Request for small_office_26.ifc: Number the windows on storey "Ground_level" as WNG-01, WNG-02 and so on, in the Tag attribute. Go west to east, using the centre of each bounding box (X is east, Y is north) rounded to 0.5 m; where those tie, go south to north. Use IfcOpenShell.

First a look at what the model holds.

```python
import ifcopenshell
import ifcopenshell.util.element
import ifcopenshell.util.placement

model = ifcopenshell.open("small_office_26.ifc")
print(model.schema)
storey = next(s for s in model.by_type("IfcBuildingStorey") if s.Name == "Ground_level")
windows = [e for e in ifcopenshell.util.element.get_decomposition(storey) if e.is_a("IfcWindow")]
for e in sorted(windows, key=lambda e: e.id()):
    origin = ifcopenshell.util.placement.get_local_placement(e.ObjectPlacement)[:3, 3]
    print(e.id(), e.Tag, e.Name, origin.round(2) + 0.0, sep=" | ")
```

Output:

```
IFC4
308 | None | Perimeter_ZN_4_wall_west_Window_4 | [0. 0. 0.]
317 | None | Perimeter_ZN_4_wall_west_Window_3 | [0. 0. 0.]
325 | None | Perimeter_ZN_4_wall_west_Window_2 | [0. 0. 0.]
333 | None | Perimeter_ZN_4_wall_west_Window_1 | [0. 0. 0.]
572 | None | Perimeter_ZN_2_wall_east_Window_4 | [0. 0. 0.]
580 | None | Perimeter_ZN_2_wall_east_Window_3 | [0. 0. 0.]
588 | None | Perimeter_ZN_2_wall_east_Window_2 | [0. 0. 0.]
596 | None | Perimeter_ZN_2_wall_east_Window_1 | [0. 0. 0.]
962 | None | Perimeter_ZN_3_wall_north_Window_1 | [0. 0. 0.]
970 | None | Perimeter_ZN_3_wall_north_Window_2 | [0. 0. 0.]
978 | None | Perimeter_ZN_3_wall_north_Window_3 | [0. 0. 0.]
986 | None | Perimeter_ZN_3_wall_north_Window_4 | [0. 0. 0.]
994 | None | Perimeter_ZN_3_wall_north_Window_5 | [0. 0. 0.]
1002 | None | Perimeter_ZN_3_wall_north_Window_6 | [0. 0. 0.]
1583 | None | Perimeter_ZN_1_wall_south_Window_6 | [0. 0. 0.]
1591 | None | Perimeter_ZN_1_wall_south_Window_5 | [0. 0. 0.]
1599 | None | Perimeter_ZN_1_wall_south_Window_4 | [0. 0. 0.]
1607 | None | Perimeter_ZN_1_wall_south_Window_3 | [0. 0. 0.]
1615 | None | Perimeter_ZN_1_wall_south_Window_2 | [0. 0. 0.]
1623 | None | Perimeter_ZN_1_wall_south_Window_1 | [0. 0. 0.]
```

```python
import ifcopenshell
import ifcopenshell.geom
import ifcopenshell.util.element
import ifcopenshell.util.shape

model = ifcopenshell.open("small_office_26.ifc")
settings = ifcopenshell.geom.settings()
settings.set("use-world-coords", True)


def centre(element):
    shape = ifcopenshell.geom.create_shape(settings, element)
    return ifcopenshell.util.shape.get_bbox_centroid(shape.geometry)


storey = next(s for s in model.by_type("IfcBuildingStorey") if s.Name == "Ground_level")
windows = [e for e in ifcopenshell.util.element.get_decomposition(storey) if e.is_a("IfcWindow")]

# Insertion points can sit at a corner or the storey origin, so sort by the geometry (in metres).
centres = {e: centre(e) for e in windows}
windows.sort(key=lambda e: (round(centres[e][0] / 0.5), centres[e][1]))

for i, e in enumerate(windows, start=1):
    number = f"WNG-{i:02d}"
    e.Tag = number
    print(e.id(), number)

model.write("small_office_26-out.ifc")
```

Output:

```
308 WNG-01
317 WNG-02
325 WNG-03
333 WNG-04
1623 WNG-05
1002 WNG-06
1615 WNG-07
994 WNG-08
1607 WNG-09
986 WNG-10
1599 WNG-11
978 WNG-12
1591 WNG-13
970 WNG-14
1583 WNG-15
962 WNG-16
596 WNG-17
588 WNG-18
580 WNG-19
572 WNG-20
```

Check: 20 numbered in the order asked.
